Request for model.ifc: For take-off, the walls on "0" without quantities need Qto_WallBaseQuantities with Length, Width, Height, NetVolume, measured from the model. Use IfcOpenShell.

First a look at what the model holds.

```python
import ifcopenshell
import ifcopenshell.util.element
import ifcopenshell.util.unit

model = ifcopenshell.open("model.ifc")
print(model.schema)
for unit_type in ("LENGTHUNIT", "AREAUNIT", "VOLUMEUNIT"):
    print(unit_type, ifcopenshell.util.unit.calculate_unit_scale(model, unit_type))
storey = next(s for s in model.by_type("IfcBuildingStorey") if s.Name == "0")
walls = [e for e in ifcopenshell.util.element.get_decomposition(storey) if e.is_a("IfcWall")]
for e in sorted(walls, key=lambda e: e.id()):
    print(e.id(), e.is_a(), e.Name, list(ifcopenshell.util.element.get_psets(e, qtos_only=True)), sep=" | ")
```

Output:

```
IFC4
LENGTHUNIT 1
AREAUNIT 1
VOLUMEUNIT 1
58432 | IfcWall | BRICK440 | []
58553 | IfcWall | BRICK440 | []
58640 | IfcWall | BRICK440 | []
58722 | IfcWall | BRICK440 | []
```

```python
import ifcopenshell
import ifcopenshell.api.pset
import ifcopenshell.geom
import ifcopenshell.util.element
import ifcopenshell.util.shape
import ifcopenshell.util.unit

model = ifcopenshell.open("model.ifc")
unit_scale = ifcopenshell.util.unit.calculate_unit_scale(model)
volume_scale = ifcopenshell.util.unit.calculate_unit_scale(model, "VOLUMEUNIT")
settings = ifcopenshell.geom.settings()

storey = next(s for s in model.by_type("IfcBuildingStorey") if s.Name == "0")
walls = [e for e in ifcopenshell.util.element.get_decomposition(storey) if e.is_a("IfcWall")]

for e in sorted(walls, key=lambda e: e.id()):
    if ifcopenshell.util.element.get_psets(e, qtos_only=True, should_inherit=False):
        continue
    # Geometry comes back in metres, in the element's own axes.
    shape = ifcopenshell.geom.create_shape(settings, e)
    values = {
        "Length": ifcopenshell.util.shape.get_x(shape.geometry) / unit_scale,
        "Width": ifcopenshell.util.shape.get_y(shape.geometry) / unit_scale,
        "Height": ifcopenshell.util.shape.get_z(shape.geometry) / unit_scale,
        "NetVolume": ifcopenshell.util.shape.get_volume(shape.geometry) / volume_scale,
    }
    qto = ifcopenshell.api.pset.add_qto(model, product=e, name="Qto_WallBaseQuantities")
    ifcopenshell.api.pset.edit_qto(model, qto=qto, properties=values)
    print(e.id(), {k: round(v, 3) for k, v in values.items()})

model.write("model_updated.ifc")
```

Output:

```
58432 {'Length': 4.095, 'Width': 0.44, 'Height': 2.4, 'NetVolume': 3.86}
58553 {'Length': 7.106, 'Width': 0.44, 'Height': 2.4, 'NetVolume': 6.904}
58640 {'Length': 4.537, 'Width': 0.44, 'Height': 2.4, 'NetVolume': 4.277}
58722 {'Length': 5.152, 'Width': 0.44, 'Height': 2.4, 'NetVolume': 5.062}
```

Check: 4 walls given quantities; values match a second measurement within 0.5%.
